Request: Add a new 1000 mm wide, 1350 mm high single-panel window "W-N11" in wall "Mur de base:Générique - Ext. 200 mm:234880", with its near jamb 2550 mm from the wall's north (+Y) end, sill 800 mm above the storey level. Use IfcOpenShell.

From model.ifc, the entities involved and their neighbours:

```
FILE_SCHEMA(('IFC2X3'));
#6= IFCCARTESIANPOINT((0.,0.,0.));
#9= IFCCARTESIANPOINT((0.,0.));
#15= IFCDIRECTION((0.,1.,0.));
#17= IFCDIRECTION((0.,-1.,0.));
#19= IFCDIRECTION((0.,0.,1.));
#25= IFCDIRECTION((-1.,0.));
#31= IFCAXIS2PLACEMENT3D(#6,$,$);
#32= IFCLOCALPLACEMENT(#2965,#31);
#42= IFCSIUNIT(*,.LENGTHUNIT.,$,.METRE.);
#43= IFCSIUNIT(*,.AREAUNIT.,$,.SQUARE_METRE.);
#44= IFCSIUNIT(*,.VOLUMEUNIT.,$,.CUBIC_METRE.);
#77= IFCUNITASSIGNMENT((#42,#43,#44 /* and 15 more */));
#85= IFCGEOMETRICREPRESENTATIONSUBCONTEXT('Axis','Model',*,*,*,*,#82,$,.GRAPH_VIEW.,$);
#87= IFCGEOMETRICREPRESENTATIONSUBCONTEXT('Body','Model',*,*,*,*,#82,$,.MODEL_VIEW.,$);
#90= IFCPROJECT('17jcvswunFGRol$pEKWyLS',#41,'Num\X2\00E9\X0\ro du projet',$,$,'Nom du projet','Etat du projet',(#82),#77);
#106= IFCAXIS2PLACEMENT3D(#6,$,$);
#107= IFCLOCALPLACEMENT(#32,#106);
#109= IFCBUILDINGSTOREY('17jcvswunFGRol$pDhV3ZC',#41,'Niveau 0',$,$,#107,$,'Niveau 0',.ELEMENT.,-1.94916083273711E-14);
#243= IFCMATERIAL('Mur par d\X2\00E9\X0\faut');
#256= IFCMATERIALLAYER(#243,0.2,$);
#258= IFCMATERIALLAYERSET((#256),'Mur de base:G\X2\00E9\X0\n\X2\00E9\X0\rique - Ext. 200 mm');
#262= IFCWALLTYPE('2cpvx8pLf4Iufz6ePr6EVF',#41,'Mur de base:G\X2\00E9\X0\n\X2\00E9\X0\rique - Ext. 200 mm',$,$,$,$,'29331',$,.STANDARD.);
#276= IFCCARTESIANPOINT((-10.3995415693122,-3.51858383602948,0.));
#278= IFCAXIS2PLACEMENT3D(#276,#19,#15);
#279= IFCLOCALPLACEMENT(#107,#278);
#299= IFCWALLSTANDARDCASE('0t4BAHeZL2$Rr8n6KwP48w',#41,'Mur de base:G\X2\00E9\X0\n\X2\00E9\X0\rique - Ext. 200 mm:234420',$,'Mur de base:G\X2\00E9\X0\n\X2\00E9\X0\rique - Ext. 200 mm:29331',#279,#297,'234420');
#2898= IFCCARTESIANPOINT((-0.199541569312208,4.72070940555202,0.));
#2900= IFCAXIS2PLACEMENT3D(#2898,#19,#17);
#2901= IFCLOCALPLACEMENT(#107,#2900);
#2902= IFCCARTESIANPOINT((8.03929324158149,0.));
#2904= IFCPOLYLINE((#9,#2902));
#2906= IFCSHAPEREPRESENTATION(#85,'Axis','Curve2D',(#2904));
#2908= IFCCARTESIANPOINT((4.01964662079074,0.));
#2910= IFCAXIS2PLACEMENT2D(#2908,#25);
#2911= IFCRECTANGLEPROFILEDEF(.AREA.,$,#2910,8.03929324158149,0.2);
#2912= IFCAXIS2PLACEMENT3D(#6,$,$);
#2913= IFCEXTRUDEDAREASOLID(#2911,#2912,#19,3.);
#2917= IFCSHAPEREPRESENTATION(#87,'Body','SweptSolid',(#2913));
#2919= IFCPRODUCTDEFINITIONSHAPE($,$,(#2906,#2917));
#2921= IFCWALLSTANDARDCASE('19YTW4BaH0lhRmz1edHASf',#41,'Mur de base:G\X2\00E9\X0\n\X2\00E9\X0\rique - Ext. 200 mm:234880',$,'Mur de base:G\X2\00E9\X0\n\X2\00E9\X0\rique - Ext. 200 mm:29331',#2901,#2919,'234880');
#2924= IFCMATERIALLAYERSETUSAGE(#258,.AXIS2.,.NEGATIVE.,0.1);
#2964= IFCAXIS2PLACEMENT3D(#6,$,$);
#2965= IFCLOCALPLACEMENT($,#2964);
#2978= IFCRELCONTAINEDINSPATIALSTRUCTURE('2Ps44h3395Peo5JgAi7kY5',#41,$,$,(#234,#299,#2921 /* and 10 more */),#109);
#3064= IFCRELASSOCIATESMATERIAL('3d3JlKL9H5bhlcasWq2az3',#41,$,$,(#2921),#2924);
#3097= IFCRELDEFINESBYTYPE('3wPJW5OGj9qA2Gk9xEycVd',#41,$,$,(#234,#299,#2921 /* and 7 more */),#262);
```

```python
import numpy as np
import ifcopenshell
import ifcopenshell.api.feature
import ifcopenshell.api.geometry
import ifcopenshell.api.root
import ifcopenshell.api.spatial
import ifcopenshell.api.type
import ifcopenshell.geom
import ifcopenshell.util.element
import ifcopenshell.util.placement
import ifcopenshell.util.representation
import ifcopenshell.util.shape
import ifcopenshell.util.unit

model = ifcopenshell.open("model.ifc")
unit_scale = ifcopenshell.util.unit.calculate_unit_scale(model)
settings = ifcopenshell.geom.settings()


def volume(element):
    """Net volume in cubic metres, openings subtracted."""
    shape = ifcopenshell.geom.create_shape(settings, element)
    return ifcopenshell.util.shape.get_volume(shape.geometry)


wall = model.by_guid("19YTW4BaH0lhRmz1edHASf")
storey = ifcopenshell.util.element.get_container(wall, ifc_class="IfcBuildingStorey")
context = ifcopenshell.util.representation.get_context(model, "Model", "Body", "MODEL_VIEW")
before = volume(wall)

width, height, from_end, sill = 1, 1.35, 2.55, 0.8  # metres

# The wall runs along its own X axis, and the end named is its -X end.
wall_shape = ifcopenshell.geom.create_shape(settings, wall)
x, y, z = ifcopenshell.util.shape.get_vertices(wall_shape.geometry).T
start = x.min() + from_end
face, thickness = float(y.min()), float(y.max() - y.min())
wall_matrix = ifcopenshell.util.placement.get_local_placement(wall.ObjectPlacement)
level = ifcopenshell.util.placement.get_local_placement(storey.ObjectPlacement)[2, 3]


def in_wall(x, y):
    """Placement at x, y metres in the wall's axes, at sill height."""
    matrix = wall_matrix.copy()
    matrix[:, 3] = wall_matrix @ np.array([x / unit_scale, y / unit_scale, 0.0, 1.0])
    matrix[2, 3] = level + sill / unit_scale
    return matrix


# Opening: a box that overshoots both wall faces by 50 mm.
opening = ifcopenshell.api.root.create_entity(model, ifc_class="IfcOpeningElement")
box = ifcopenshell.api.geometry.add_wall_representation(
    model, context=context, length=width, height=height, thickness=thickness + 0.1
)
ifcopenshell.api.geometry.assign_representation(model, product=opening, representation=box)
ifcopenshell.api.geometry.edit_object_placement(model, product=opening, matrix=in_wall(start, face - 0.05), is_si=False)
ifcopenshell.api.feature.add_feature(model, feature=opening, element=wall)

window = ifcopenshell.api.root.create_entity(model, ifc_class="IfcWindow", name="W-N11")
window.OverallWidth, window.OverallHeight = width / unit_scale, height / unit_scale
body = ifcopenshell.api.geometry.add_window_representation(
    model,
    context=context,
    overall_width=window.OverallWidth,
    overall_height=window.OverallHeight,
    partition_type="SINGLE_PANEL",
)
ifcopenshell.api.geometry.assign_representation(model, product=window, representation=body)
ifcopenshell.api.spatial.assign_container(model, products=[window], relating_structure=storey)
fills = ifcopenshell.api.feature.add_filling(model, opening=opening, element=window)
fills.OwnerHistory = window.OwnerHistory  # required in IFC2X3

# IFC2X3 keeps the operation on the window style.
style = ifcopenshell.api.root.create_entity(model, ifc_class="IfcWindowStyle", name="W-N11")
style.OperationType, style.ConstructionType = "SINGLE_PANEL", "NOTDEFINED"
style.ParameterTakesPrecedence = style.Sizeable = False
ifcopenshell.api.type.assign_type(model, related_objects=[window], relating_type=style)

# Centre the window in the wall's thickness.
ifcopenshell.api.geometry.edit_object_placement(model, product=window, matrix=in_wall(start, face), is_si=False)
window_shape = ifcopenshell.geom.create_shape(settings, window)
depth = ifcopenshell.util.shape.get_vertices(window_shape.geometry)[:, 1]
offset = face + thickness / 2 - (depth.min() + depth.max()) / 2
ifcopenshell.api.geometry.edit_object_placement(model, product=window, matrix=in_wall(start, offset), is_si=False)

after = volume(wall)

print(f"wall volume {before:.3f} -> {after:.3f} m3")

model.write("model_updated.ifc")
```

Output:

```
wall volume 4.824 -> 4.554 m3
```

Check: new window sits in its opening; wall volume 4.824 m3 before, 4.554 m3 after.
